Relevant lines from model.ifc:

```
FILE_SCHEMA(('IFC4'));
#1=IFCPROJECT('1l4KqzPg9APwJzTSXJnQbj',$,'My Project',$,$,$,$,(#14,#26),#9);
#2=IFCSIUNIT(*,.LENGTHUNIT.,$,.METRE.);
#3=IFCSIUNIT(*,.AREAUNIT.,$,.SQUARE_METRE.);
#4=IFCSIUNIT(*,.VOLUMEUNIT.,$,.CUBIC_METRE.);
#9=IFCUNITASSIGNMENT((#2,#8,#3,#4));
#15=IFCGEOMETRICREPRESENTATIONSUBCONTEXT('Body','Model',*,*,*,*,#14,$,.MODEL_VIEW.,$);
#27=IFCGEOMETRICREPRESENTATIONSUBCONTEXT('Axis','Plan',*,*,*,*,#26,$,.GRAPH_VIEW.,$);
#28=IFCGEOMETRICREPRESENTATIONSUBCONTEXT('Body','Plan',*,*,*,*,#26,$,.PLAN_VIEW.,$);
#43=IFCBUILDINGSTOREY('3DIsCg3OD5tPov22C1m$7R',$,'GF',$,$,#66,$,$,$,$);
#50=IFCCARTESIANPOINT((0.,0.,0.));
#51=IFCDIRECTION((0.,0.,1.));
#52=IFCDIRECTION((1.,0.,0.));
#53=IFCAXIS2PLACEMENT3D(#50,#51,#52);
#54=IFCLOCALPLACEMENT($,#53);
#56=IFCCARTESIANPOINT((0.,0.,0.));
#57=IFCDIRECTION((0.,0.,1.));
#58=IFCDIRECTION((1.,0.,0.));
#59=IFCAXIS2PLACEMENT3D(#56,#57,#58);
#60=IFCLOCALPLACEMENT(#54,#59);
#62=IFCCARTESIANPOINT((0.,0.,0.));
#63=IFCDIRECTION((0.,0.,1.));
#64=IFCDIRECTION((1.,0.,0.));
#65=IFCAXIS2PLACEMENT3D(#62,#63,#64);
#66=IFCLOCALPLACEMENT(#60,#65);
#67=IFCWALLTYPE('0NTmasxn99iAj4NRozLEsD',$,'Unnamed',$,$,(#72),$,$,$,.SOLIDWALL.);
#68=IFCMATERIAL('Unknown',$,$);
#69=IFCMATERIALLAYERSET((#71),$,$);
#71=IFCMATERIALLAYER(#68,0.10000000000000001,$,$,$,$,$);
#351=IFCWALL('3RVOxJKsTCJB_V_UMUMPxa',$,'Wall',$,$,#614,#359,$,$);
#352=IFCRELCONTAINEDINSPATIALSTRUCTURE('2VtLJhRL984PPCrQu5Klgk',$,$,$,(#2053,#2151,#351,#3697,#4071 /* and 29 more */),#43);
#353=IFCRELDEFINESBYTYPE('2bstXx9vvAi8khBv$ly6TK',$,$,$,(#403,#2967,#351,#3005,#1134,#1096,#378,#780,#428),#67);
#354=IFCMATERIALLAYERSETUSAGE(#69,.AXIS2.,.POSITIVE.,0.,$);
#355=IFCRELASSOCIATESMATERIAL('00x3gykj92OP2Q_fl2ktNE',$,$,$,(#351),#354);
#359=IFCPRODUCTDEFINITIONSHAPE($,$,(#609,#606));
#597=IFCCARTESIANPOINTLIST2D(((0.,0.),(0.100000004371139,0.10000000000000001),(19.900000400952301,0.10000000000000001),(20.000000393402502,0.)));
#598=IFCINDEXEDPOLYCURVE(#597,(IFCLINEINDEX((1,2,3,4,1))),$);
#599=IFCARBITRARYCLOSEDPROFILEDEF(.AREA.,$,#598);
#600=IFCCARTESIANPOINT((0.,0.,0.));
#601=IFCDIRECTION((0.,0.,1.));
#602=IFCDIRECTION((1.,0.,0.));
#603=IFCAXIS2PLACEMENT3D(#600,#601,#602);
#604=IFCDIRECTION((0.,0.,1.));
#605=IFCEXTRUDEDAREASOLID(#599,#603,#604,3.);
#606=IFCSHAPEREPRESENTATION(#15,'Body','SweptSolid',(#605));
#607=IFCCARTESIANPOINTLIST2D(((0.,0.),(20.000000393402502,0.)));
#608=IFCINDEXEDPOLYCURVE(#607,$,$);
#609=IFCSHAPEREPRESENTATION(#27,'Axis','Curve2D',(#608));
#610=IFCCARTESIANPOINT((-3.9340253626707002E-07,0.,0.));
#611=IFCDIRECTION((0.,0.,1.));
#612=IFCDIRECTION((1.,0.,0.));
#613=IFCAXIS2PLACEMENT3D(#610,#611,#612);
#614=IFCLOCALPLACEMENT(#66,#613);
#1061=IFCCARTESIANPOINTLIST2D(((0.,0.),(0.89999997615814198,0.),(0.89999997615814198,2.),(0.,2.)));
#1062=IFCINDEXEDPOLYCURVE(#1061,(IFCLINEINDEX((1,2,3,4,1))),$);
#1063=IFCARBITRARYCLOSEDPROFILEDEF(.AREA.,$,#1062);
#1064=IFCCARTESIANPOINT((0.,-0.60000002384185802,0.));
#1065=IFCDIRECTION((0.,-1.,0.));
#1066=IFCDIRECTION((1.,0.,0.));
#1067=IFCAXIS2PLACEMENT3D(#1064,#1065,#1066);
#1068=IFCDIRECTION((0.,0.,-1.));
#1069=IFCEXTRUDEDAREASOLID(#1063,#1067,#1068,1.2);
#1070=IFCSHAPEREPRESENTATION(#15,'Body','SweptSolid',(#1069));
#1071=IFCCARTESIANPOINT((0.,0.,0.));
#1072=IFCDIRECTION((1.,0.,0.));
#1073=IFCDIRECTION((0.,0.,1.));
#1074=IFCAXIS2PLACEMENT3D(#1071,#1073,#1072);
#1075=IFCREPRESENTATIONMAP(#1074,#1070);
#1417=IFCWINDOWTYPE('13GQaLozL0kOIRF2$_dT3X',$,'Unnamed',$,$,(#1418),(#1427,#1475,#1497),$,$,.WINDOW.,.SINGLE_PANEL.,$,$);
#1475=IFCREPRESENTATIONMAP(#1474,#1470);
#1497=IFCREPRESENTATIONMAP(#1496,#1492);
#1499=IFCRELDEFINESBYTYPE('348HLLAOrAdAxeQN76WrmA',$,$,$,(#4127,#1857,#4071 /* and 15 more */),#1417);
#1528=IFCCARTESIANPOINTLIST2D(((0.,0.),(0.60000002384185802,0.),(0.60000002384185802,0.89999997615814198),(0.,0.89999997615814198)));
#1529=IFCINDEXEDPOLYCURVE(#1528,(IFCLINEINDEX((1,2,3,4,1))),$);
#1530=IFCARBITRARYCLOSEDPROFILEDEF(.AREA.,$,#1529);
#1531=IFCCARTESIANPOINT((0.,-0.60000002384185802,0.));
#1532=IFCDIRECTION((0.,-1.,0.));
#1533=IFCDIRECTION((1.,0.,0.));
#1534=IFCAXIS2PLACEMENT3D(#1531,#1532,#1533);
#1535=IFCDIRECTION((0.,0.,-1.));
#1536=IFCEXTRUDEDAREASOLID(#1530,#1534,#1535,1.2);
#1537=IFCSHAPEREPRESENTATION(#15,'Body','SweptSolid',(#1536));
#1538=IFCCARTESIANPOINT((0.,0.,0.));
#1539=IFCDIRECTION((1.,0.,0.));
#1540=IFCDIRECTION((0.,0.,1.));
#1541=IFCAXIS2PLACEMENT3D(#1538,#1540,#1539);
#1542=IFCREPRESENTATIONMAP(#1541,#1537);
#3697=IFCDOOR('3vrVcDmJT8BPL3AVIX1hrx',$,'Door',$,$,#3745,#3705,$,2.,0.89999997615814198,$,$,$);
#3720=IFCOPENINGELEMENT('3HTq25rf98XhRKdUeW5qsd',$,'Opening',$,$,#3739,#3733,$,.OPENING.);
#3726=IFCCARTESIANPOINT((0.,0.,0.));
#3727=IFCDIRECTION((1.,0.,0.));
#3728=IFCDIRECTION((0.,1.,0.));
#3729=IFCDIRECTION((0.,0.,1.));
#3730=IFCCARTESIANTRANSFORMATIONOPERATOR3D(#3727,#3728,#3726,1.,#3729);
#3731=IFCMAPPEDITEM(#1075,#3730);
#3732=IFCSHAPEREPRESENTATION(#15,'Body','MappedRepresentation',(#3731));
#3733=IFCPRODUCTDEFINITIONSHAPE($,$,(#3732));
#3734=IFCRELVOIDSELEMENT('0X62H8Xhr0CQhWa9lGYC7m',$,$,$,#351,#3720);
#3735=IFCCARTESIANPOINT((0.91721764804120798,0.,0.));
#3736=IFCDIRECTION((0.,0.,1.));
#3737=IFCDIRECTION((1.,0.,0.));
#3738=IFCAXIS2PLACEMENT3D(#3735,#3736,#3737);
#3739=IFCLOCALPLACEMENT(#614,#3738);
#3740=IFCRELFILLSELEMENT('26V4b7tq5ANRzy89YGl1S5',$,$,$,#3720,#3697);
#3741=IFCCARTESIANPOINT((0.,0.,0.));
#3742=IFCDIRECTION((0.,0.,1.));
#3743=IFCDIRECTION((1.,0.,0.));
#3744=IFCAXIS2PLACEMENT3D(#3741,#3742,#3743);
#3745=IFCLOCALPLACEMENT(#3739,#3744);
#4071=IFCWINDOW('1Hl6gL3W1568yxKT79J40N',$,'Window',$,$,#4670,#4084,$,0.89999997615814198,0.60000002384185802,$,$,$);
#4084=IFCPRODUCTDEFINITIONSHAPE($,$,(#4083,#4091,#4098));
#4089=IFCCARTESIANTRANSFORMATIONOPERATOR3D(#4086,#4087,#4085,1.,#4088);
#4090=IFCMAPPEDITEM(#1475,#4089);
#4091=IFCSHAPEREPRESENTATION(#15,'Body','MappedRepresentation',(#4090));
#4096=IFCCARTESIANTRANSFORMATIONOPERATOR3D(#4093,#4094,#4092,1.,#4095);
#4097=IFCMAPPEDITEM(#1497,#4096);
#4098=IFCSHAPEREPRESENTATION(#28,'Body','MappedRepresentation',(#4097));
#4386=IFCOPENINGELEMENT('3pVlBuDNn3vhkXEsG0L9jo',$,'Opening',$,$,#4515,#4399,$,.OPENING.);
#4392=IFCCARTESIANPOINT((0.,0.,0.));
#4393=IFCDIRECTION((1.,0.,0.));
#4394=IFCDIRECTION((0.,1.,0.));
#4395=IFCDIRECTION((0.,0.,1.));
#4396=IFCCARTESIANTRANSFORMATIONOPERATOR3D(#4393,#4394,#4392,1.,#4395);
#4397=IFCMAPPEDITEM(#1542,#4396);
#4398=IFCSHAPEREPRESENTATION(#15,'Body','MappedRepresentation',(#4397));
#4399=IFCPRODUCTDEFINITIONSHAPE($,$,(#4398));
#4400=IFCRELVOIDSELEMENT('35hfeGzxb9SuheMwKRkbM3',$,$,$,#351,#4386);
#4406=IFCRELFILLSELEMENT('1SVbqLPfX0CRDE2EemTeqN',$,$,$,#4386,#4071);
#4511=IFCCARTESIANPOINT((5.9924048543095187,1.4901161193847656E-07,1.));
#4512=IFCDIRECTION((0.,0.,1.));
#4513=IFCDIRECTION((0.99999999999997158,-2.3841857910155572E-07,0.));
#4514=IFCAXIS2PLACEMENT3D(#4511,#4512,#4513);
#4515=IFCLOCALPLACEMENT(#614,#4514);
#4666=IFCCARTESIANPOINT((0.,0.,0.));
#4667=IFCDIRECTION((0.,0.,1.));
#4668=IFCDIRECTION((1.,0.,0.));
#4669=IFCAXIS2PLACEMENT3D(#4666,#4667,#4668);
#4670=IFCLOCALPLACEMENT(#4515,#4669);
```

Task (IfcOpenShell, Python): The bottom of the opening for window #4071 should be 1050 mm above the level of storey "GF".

```python
import numpy as np
import ifcopenshell
import ifcopenshell.api.geometry
import ifcopenshell.geom
import ifcopenshell.util.element
import ifcopenshell.util.placement
import ifcopenshell.util.shape
import ifcopenshell.util.unit

model = ifcopenshell.open("model.ifc")
unit_scale = ifcopenshell.util.unit.calculate_unit_scale(model)

window = model.by_guid("1Hl6gL3W1568yxKT79J40N")
opening = window.FillsVoids[0].RelatingOpeningElement
storey = ifcopenshell.util.element.get_container(window, ifc_class="IfcBuildingStorey")
level = ifcopenshell.util.placement.get_local_placement(storey.ObjectPlacement)[2, 3]

# The opening's origin need not be at the sill, so measure its lowest point.
shape = ifcopenshell.geom.create_shape(ifcopenshell.geom.settings(), opening)
bottom = ifcopenshell.util.shape.get_shape_bottom_elevation(shape, shape.geometry) / unit_scale
dz = level + 1.05 - bottom

shift = np.array([0.0, 0.0, dz])
# The window is placed relative to its opening, so it follows when the opening moves.
matrix = ifcopenshell.util.placement.get_local_placement(opening.ObjectPlacement)
matrix[:3, 3] += shift
ifcopenshell.api.geometry.edit_object_placement(
    model, product=opening, matrix=matrix, is_si=False, should_transform_children=True
)

print(f"moved by {dz * unit_scale:+.3f} m")

model.write("model_v2.ifc")
```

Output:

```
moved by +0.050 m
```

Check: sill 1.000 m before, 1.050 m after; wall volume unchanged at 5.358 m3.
